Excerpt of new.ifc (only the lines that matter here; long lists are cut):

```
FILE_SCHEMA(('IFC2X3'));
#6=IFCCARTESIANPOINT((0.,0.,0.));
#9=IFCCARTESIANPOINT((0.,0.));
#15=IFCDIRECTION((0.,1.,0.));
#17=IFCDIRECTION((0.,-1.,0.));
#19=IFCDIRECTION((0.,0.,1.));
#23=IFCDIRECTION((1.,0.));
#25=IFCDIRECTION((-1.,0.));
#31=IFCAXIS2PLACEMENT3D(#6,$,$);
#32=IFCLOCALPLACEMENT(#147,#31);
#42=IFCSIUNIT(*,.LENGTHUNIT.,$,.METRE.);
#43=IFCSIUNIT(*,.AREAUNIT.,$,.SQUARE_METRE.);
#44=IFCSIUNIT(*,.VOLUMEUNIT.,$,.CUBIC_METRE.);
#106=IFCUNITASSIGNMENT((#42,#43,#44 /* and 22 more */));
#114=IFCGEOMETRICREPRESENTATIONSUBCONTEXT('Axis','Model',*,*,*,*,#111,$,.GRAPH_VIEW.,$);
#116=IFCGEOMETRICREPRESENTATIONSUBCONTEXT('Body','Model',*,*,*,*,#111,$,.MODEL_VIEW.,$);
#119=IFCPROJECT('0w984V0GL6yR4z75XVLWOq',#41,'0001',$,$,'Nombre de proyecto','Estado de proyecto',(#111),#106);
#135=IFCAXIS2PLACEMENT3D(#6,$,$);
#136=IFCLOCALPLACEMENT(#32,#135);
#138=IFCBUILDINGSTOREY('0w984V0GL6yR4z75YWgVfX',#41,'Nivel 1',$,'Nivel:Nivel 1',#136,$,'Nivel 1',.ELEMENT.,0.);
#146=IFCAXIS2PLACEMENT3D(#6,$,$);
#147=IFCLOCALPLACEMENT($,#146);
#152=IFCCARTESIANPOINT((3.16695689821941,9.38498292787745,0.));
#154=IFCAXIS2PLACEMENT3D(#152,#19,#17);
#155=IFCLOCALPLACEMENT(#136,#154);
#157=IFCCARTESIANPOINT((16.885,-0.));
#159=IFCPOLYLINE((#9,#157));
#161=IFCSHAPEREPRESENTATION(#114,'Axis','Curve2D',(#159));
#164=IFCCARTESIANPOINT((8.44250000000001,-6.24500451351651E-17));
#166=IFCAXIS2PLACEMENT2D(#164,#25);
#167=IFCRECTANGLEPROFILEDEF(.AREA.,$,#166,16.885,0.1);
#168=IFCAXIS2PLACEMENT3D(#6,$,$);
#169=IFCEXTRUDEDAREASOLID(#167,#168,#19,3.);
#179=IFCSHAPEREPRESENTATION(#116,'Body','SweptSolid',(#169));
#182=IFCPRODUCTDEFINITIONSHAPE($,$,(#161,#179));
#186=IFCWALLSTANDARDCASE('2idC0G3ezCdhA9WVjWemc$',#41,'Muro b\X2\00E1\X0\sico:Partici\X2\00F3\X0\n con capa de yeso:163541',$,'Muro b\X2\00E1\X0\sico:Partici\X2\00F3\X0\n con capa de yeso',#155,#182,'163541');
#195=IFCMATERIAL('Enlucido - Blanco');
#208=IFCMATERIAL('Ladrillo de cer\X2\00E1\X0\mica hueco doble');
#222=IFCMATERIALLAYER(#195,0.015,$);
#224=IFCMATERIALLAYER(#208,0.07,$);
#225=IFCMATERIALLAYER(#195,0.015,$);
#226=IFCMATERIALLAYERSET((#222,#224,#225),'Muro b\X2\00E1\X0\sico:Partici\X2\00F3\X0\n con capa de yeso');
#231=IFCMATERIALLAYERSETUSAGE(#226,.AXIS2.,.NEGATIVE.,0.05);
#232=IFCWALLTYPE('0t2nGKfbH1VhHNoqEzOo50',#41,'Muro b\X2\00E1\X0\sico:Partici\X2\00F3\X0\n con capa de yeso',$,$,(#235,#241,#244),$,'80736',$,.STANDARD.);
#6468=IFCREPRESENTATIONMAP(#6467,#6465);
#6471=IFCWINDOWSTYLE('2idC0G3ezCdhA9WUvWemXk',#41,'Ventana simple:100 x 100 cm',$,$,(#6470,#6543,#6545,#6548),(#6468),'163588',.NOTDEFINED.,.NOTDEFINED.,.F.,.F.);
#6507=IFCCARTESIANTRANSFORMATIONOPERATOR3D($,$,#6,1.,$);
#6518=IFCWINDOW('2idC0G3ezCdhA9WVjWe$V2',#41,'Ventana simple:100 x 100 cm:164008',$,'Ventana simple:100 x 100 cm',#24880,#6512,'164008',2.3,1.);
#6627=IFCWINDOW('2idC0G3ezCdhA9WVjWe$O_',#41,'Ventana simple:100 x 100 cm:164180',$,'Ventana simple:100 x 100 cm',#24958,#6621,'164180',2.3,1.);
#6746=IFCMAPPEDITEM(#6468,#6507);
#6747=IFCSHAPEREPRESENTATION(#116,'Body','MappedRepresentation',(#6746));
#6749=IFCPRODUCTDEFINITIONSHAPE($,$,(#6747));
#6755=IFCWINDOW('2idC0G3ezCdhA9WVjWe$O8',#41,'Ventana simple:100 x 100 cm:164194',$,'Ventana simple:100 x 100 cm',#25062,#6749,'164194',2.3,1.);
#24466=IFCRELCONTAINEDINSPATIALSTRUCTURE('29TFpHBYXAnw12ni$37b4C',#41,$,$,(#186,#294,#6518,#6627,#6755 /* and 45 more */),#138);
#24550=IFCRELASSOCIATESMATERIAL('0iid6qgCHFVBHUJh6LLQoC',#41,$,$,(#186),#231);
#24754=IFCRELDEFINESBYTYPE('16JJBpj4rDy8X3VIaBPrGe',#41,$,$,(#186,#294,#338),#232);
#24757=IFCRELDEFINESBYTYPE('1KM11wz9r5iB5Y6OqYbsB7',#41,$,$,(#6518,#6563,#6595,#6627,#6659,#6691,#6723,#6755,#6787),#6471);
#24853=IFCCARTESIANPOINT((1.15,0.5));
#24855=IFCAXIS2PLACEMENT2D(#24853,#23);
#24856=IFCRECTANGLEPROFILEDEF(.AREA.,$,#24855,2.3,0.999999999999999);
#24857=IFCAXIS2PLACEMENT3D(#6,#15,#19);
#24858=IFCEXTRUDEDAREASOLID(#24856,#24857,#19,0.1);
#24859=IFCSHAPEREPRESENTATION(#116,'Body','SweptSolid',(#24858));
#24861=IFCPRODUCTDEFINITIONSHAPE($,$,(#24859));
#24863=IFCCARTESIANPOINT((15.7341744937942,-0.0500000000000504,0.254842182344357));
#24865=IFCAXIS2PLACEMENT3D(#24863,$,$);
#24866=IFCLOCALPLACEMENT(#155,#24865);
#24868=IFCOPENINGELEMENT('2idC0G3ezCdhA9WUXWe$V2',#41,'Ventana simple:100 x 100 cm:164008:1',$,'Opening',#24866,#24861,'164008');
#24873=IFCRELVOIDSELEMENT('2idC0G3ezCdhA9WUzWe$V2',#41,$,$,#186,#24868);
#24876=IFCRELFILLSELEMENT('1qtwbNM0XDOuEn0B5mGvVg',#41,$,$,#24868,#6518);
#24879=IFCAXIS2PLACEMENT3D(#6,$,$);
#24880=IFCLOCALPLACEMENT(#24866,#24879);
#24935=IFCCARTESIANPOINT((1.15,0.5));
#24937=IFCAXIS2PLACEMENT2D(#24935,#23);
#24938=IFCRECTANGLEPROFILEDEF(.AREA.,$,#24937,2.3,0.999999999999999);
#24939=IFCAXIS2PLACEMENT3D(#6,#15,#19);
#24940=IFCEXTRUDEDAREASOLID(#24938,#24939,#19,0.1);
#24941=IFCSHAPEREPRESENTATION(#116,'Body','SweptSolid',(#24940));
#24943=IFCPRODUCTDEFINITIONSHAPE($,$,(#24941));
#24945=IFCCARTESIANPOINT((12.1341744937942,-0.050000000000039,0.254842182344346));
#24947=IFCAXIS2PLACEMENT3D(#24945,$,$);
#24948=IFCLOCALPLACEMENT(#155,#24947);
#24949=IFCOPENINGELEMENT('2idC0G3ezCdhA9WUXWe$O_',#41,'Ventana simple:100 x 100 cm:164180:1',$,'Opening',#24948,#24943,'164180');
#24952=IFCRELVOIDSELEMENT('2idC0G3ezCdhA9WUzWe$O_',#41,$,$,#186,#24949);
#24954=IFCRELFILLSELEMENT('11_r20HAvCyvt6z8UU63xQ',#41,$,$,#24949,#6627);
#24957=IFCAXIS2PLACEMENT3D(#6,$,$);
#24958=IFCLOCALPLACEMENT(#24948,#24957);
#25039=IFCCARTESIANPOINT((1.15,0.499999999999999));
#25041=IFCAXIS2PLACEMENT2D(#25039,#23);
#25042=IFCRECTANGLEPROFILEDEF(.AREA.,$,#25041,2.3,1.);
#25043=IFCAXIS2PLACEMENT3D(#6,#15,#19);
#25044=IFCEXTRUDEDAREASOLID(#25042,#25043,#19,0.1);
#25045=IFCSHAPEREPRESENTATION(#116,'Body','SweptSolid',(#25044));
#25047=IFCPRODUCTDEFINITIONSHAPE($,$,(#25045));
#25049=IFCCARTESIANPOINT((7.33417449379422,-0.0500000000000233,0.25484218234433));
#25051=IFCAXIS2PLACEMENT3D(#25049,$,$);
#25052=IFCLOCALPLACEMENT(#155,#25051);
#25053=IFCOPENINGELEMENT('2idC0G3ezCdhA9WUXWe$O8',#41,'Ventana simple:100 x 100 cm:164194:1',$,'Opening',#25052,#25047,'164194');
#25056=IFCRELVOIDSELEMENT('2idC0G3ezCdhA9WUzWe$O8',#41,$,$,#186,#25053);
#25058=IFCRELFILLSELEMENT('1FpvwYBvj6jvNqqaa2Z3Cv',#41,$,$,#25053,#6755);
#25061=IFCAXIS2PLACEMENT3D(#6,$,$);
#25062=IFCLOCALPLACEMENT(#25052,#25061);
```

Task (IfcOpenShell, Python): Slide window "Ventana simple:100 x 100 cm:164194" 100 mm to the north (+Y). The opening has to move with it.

```python
import ifcopenshell
import ifcopenshell.api.geometry
import ifcopenshell.util.placement
import ifcopenshell.util.unit

model = ifcopenshell.open("new.ifc")
unit_scale = ifcopenshell.util.unit.calculate_unit_scale(model)

window = model.by_guid("2idC0G3ezCdhA9WVjWe$O8")
opening = window.FillsVoids[0].RelatingOpeningElement
wall = opening.VoidsElements[0].RelatingBuildingElement

wall_matrix = ifcopenshell.util.placement.get_local_placement(wall.ObjectPlacement)
shift = wall_matrix[:3, 0] * -0.1 / unit_scale
before = ifcopenshell.util.placement.get_local_placement(window.ObjectPlacement)[:3, 3].copy()

# The window is placed relative to its opening, so it follows when the opening moves.
matrix = ifcopenshell.util.placement.get_local_placement(opening.ObjectPlacement)
matrix[:3, 3] += shift
ifcopenshell.api.geometry.edit_object_placement(
    model, product=opening, matrix=matrix, is_si=False, should_transform_children=True
)

after = ifcopenshell.util.placement.get_local_placement(window.ObjectPlacement)[:3, 3]
print("window moved by", (after - before).round(3) + 0.0)

model.write("new_edited.ifc")
```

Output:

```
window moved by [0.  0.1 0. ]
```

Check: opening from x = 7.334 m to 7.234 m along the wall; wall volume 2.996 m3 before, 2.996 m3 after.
